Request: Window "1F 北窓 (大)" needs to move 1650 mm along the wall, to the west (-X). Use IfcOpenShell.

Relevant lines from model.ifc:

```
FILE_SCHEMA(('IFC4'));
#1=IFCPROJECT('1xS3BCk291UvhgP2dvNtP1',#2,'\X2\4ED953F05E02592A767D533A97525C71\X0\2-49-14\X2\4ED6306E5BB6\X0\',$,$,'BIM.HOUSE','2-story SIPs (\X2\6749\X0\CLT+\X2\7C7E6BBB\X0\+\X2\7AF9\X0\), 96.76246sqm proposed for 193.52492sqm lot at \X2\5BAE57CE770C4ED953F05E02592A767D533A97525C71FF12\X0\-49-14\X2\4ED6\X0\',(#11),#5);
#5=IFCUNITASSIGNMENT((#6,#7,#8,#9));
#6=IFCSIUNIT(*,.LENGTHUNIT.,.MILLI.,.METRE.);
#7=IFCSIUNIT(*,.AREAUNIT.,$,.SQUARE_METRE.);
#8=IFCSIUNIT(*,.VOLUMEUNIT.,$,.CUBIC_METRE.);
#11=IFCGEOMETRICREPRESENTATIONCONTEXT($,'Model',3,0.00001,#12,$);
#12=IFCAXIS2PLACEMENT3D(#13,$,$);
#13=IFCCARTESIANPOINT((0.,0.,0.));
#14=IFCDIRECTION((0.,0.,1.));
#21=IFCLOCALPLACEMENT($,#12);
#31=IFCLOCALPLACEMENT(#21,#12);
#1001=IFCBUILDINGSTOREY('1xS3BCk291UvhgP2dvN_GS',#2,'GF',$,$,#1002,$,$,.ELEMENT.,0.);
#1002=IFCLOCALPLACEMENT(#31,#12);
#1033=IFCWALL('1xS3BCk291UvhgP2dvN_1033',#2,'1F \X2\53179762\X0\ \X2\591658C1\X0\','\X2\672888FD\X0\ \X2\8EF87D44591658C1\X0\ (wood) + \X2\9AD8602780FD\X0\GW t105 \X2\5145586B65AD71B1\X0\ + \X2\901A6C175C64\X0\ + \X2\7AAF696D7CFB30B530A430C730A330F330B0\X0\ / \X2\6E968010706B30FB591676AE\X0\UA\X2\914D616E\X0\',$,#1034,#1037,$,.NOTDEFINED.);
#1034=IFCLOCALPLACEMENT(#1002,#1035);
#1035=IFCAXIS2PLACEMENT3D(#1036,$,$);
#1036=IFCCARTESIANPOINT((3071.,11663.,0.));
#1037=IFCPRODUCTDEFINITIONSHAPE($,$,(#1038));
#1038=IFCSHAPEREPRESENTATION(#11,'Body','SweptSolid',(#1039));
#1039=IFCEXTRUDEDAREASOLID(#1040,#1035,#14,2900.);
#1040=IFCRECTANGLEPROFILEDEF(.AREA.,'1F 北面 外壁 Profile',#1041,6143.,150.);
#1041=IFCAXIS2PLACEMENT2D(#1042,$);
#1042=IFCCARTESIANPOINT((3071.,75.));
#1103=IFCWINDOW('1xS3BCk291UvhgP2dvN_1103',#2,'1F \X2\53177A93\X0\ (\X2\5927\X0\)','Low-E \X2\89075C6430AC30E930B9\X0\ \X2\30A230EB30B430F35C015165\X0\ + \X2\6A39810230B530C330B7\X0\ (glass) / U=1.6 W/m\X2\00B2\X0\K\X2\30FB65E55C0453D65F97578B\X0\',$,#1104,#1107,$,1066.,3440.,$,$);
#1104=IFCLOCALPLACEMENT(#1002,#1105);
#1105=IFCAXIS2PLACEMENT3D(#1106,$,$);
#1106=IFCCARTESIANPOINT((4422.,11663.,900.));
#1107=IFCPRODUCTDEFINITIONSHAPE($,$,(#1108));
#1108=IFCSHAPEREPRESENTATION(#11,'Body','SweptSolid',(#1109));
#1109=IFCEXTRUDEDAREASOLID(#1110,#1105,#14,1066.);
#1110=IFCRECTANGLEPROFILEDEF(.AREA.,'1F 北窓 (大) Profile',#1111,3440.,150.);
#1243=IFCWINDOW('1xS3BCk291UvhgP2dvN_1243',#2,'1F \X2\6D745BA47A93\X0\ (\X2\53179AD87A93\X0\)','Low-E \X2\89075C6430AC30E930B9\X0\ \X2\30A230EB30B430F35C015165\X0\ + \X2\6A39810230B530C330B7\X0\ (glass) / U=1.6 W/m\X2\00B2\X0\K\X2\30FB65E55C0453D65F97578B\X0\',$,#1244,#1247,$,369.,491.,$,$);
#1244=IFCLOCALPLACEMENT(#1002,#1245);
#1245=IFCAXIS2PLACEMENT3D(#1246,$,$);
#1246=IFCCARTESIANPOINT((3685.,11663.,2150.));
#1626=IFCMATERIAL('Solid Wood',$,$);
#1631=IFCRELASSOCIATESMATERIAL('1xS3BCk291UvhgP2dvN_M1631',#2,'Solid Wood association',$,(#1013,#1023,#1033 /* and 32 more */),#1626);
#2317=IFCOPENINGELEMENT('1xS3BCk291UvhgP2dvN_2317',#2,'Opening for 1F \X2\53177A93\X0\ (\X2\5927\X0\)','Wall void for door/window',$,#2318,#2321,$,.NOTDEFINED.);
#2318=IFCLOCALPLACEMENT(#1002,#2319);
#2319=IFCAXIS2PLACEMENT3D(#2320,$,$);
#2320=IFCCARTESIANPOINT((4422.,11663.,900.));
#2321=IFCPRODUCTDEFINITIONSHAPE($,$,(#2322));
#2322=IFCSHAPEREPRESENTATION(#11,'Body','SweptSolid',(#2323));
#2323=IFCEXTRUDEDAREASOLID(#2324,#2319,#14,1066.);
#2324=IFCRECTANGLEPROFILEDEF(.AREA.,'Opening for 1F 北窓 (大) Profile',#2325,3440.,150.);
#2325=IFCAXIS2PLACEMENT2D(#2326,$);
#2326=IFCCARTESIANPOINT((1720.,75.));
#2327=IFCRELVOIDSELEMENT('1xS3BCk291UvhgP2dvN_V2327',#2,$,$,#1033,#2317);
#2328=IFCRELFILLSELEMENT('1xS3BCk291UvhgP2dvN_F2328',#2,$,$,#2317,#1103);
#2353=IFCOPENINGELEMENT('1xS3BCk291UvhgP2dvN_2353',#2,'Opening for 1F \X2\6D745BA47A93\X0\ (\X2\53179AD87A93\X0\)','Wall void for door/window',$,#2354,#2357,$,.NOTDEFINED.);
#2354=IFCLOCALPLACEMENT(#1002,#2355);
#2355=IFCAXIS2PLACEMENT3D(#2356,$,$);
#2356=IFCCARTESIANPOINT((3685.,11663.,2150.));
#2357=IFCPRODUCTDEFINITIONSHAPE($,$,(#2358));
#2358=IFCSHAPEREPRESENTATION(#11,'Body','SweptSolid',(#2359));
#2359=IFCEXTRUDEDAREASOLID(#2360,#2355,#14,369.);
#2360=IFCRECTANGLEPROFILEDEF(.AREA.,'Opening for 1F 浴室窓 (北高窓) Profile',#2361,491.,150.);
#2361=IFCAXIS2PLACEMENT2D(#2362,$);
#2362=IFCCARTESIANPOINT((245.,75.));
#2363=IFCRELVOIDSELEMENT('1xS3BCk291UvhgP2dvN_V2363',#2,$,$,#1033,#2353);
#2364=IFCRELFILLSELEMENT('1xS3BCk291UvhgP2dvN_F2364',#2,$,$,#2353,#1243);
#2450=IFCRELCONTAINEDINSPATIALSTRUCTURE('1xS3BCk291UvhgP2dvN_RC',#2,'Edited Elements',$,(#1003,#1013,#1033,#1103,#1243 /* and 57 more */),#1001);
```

```python
import ifcopenshell
import ifcopenshell.api.geometry
import ifcopenshell.util.placement

model = ifcopenshell.open("model.ifc")

window = model.by_guid("1xS3BCk291UvhgP2dvN_1103")
opening = window.FillsVoids[0].RelatingOpeningElement
wall = opening.VoidsElements[0].RelatingBuildingElement

wall_matrix = ifcopenshell.util.placement.get_local_placement(wall.ObjectPlacement)
shift = wall_matrix[:3, 0] * -1650.0
before = ifcopenshell.util.placement.get_local_placement(window.ObjectPlacement)[:3, 3].copy()

# The window is not placed relative to its opening, so move both.
for product in (opening, window):
    matrix = ifcopenshell.util.placement.get_local_placement(product.ObjectPlacement)
    matrix[:3, 3] += shift
    ifcopenshell.api.geometry.edit_object_placement(model, product=product, matrix=matrix, is_si=False)

after = ifcopenshell.util.placement.get_local_placement(window.ObjectPlacement)[:3, 3]
print("window moved by", (after - before).round(3) + 0.0)

model.write("model_v2.ifc")
```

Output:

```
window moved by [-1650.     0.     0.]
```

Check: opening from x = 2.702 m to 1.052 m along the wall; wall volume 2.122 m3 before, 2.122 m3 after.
